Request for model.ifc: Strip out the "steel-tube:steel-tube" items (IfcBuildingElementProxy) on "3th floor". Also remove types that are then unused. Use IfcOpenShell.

First a look at what the model holds.

```python
import ifcopenshell
import ifcopenshell.util.element

model = ifcopenshell.open("model.ifc")
print(model.schema)
storey = next(s for s in model.by_type("IfcBuildingStorey") if s.Name == "3th floor")
proxies = [e for e in ifcopenshell.util.element.get_decomposition(storey) if e.is_a("IfcBuildingElementProxy")]
seen = {}
for e in proxies:
    element_type = ifcopenshell.util.element.get_type(e)
    name = element_type.Name if element_type not in (None, e) else None
    seen[name] = seen.get(name, 0) + 1
for name, count in sorted(seen.items(), key=str):
    print(count, "x", name)
```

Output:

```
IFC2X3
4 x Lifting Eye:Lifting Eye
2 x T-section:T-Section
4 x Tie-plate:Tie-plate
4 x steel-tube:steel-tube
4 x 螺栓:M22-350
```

```python
import ifcopenshell
import ifcopenshell.api.root
import ifcopenshell.util.element

model = ifcopenshell.open("model.ifc")

storey = next(s for s in model.by_type("IfcBuildingStorey") if s.Name == "3th floor")
proxies = [e for e in ifcopenshell.util.element.get_decomposition(storey) if e.is_a("IfcBuildingElementProxy")]
targets = [e for e in proxies if (t := ifcopenshell.util.element.get_type(e)) not in (None, e) and t.Name == "steel-tube:steel-tube"]
types = {ifcopenshell.util.element.get_type(e) for e in targets} - {None, *targets}

for e in targets:
    ifcopenshell.api.root.remove_product(model, product=e)
print(len(targets), "removed")

unused = [t for t in types if not ifcopenshell.util.element.get_types(t)]
for t in unused:
    ifcopenshell.api.root.remove_product(model, product=t)
print(len(unused), "unused types removed")

model.write("model_rev.ifc")
```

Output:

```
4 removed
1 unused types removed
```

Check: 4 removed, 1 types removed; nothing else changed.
